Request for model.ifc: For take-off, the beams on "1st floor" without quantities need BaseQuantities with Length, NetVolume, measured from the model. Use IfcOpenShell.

First a look at what the model holds.

```python
import ifcopenshell
import ifcopenshell.util.element
import ifcopenshell.util.unit

model = ifcopenshell.open("model.ifc")
print(model.schema)
for unit_type in ("LENGTHUNIT", "AREAUNIT", "VOLUMEUNIT"):
    print(unit_type, ifcopenshell.util.unit.calculate_unit_scale(model, unit_type))
storey = next(s for s in model.by_type("IfcBuildingStorey") if s.Name == "1st floor")
beams = [e for e in ifcopenshell.util.element.get_decomposition(storey) if e.is_a("IfcBeam")]
for e in sorted(beams, key=lambda e: e.id()):
    print(e.id(), e.is_a(), e.Name, list(ifcopenshell.util.element.get_psets(e, qtos_only=True)), sep=" | ")
```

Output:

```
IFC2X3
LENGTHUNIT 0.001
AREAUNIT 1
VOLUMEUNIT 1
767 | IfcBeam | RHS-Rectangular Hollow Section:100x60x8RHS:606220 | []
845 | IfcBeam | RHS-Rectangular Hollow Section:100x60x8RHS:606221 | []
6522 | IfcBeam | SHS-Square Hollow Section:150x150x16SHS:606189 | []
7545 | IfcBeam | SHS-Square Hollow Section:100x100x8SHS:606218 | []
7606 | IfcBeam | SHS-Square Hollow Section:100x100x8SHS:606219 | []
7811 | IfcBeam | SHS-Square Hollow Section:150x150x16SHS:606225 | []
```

```python
import ifcopenshell
import ifcopenshell.api.pset
import ifcopenshell.geom
import ifcopenshell.util.element
import ifcopenshell.util.shape
import ifcopenshell.util.unit

model = ifcopenshell.open("model.ifc")
unit_scale = ifcopenshell.util.unit.calculate_unit_scale(model)
volume_scale = ifcopenshell.util.unit.calculate_unit_scale(model, "VOLUMEUNIT")
settings = ifcopenshell.geom.settings()

storey = next(s for s in model.by_type("IfcBuildingStorey") if s.Name == "1st floor")
beams = [e for e in ifcopenshell.util.element.get_decomposition(storey) if e.is_a("IfcBeam")]

for e in sorted(beams, key=lambda e: e.id()):
    if ifcopenshell.util.element.get_psets(e, qtos_only=True, should_inherit=False):
        continue
    # Geometry comes back in metres, in the element's own axes.
    shape = ifcopenshell.geom.create_shape(settings, e)
    values = {
        "Length": ifcopenshell.util.shape.get_max_xyz(shape.geometry) / unit_scale,
        "NetVolume": ifcopenshell.util.shape.get_volume(shape.geometry) / volume_scale,
    }
    qto = ifcopenshell.api.pset.add_qto(model, product=e, name="BaseQuantities")
    ifcopenshell.api.pset.edit_qto(model, qto=qto, properties=values)
    print(e.id(), {k: round(v, 3) for k, v in values.items()})

model.write("model_updated.ifc")
```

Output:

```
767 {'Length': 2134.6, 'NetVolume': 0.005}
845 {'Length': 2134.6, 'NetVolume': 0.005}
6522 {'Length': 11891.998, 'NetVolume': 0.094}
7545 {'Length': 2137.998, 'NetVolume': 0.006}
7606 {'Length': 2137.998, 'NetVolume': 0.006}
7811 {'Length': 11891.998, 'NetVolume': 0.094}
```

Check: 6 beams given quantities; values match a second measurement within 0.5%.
